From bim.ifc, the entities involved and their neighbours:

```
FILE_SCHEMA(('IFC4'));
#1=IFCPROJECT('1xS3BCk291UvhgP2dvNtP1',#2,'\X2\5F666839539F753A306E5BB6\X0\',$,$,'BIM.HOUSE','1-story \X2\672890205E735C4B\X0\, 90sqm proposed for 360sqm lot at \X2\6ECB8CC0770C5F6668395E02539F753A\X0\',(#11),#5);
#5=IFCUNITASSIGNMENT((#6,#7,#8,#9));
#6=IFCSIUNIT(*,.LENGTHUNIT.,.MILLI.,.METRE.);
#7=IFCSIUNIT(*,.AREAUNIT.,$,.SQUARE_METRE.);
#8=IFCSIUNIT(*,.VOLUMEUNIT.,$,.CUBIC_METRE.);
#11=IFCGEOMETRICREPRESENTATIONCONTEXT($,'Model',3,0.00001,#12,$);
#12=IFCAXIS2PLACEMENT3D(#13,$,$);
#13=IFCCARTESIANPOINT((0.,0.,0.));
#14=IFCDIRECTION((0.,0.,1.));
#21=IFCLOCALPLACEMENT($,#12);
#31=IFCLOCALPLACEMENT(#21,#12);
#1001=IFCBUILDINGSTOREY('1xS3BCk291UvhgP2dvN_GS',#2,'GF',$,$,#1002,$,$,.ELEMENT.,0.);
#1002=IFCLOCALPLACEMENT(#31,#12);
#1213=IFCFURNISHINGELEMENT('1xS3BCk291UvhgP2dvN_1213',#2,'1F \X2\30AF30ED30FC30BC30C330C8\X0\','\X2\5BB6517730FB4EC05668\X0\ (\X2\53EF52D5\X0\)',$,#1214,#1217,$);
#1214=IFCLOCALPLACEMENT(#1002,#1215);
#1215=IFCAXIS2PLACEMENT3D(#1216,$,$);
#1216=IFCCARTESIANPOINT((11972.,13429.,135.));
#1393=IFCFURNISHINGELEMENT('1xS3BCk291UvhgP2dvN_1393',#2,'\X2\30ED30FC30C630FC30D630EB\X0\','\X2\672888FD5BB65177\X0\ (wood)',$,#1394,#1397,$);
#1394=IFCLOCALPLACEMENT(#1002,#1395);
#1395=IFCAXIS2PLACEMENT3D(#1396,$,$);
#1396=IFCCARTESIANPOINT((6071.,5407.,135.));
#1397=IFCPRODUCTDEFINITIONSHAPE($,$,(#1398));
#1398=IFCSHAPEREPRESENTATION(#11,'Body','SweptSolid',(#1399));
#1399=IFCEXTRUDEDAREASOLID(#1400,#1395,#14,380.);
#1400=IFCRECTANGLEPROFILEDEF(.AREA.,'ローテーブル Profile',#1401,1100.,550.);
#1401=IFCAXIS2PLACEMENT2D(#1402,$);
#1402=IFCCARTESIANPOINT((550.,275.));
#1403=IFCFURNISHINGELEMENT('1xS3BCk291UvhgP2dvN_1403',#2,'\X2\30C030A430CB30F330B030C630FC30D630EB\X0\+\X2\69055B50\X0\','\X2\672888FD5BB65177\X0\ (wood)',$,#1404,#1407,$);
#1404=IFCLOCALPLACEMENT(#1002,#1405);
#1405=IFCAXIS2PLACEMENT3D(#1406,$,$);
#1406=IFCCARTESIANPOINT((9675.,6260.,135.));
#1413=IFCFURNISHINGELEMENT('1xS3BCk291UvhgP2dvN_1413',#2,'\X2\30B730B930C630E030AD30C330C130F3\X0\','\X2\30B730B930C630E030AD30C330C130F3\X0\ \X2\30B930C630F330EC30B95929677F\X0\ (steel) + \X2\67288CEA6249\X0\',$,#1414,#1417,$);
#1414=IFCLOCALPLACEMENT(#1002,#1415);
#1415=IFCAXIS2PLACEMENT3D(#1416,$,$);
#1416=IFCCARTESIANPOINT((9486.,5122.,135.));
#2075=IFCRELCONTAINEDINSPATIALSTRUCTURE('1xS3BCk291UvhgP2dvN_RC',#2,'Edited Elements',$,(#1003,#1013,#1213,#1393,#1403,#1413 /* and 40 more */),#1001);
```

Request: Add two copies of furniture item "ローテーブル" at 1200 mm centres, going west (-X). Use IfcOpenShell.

```python
import numpy as np
import ifcopenshell
import ifcopenshell.api.geometry
import ifcopenshell.api.root
import ifcopenshell.util.element
import ifcopenshell.util.placement
import ifcopenshell.util.unit

model = ifcopenshell.open("bim.ifc")
unit_scale = ifcopenshell.util.unit.calculate_unit_scale(model)


def reuse_history(source, copy):
    """copy_class also copies each property set's owner history, people and application; keep the originals."""
    for rel in copy.IsDefinedBy:
        if rel.is_a("IfcRelDefinesByProperties") and (history := rel.RelatingPropertyDefinition.OwnerHistory):
            rel.RelatingPropertyDefinition.OwnerHistory = source.OwnerHistory
            ifcopenshell.util.element.remove_deep2(model, history)


source = model.by_guid("1xS3BCk291UvhgP2dvN_1393")
base = ifcopenshell.util.placement.get_local_placement(source.ObjectPlacement)
step = np.array([-1.0, 0.0, 0.0]) * 1.2 / unit_scale

for i in range(1, 3):
    copy = ifcopenshell.api.root.copy_class(model, product=source)
    copy.Representation = ifcopenshell.util.element.copy_deep(
        model, source.Representation, exclude=["IfcGeometricRepresentationContext", "IfcRepresentationMap"]
    )
    reuse_history(source, copy)
    matrix = base.copy()
    matrix[:3, 3] += i * step
    print("added at", matrix[:3, 3].round(3) + 0.0)
    ifcopenshell.api.geometry.edit_object_placement(model, product=copy, matrix=matrix, is_si=False)

model.write("bim_edited.ifc")
```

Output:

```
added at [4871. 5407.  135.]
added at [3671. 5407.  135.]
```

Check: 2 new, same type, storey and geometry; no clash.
